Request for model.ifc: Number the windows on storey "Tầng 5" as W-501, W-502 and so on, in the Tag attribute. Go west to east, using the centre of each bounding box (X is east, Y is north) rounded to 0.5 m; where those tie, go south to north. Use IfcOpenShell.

First a look at what the model holds.

```python
import ifcopenshell
import ifcopenshell.util.element
import ifcopenshell.util.placement

model = ifcopenshell.open("model.ifc")
print(model.schema)
storey = next(s for s in model.by_type("IfcBuildingStorey") if s.Name == "Tầng 5")
windows = [e for e in ifcopenshell.util.element.get_decomposition(storey) if e.is_a("IfcWindow")]
for e in sorted(windows, key=lambda e: e.id()):
    origin = ifcopenshell.util.placement.get_local_placement(e.ObjectPlacement)[:3, 3]
    print(e.id(), e.Tag, e.Name, origin.round(2) + 0.0, sep=" | ")
```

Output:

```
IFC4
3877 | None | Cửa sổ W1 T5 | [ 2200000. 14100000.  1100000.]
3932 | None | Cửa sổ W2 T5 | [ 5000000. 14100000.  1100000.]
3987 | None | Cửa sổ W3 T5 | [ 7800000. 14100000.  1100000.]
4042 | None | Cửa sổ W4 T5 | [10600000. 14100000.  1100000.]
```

```python
import ifcopenshell
import ifcopenshell.geom
import ifcopenshell.util.element
import ifcopenshell.util.shape

model = ifcopenshell.open("model.ifc")
settings = ifcopenshell.geom.settings()
settings.set("use-world-coords", True)


def centre(element):
    shape = ifcopenshell.geom.create_shape(settings, element)
    return ifcopenshell.util.shape.get_bbox_centroid(shape.geometry)


storey = next(s for s in model.by_type("IfcBuildingStorey") if s.Name == "Tầng 5")
windows = [e for e in ifcopenshell.util.element.get_decomposition(storey) if e.is_a("IfcWindow")]

# Insertion points can sit at a corner or the storey origin, so sort by the geometry (in metres).
centres = {e: centre(e) for e in windows}
windows.sort(key=lambda e: (round(centres[e][0] / 0.5), centres[e][1]))

for i, e in enumerate(windows, start=1):
    number = f"W-5{i:02d}"
    e.Tag = number
    print(e.id(), number)

model.write("model_rev.ifc")
```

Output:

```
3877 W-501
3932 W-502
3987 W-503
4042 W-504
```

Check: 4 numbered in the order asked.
